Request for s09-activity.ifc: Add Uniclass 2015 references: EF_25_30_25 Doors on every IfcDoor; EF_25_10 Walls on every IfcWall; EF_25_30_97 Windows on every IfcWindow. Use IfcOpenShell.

First a look at what the model holds.

```python
import ifcopenshell

model = ifcopenshell.open("s09-activity.ifc")
print(model.schema)
print("classifications:", [c.Name for c in model.by_type("IfcClassification")])
for ifc_class in ("IfcDoor", "IfcRoof", "IfcStair", "IfcWall", "IfcWindow"):
    print(ifc_class, len(model.by_type(ifc_class)))
```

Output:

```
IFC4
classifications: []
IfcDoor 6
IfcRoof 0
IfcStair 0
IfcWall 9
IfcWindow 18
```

```python
import ifcopenshell
import ifcopenshell.api.classification

model = ifcopenshell.open("s09-activity.ifc")

system = ifcopenshell.api.classification.add_classification(model, classification="Uniclass 2015")

codes = {
    "IfcDoor": ("EF_25_30_25", "Doors"),
    "IfcWall": ("EF_25_10", "Walls"),
    "IfcWindow": ("EF_25_30_97", "Windows"),
}
for ifc_class, (code, name) in codes.items():
    products = model.by_type(ifc_class)
    ifcopenshell.api.classification.add_reference(
        model, products=products, classification=system, identification=code, name=name
    )
    print(code, len(products))

model.write("s09-activity-out.ifc")
```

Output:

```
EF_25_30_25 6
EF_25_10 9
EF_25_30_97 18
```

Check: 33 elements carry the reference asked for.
